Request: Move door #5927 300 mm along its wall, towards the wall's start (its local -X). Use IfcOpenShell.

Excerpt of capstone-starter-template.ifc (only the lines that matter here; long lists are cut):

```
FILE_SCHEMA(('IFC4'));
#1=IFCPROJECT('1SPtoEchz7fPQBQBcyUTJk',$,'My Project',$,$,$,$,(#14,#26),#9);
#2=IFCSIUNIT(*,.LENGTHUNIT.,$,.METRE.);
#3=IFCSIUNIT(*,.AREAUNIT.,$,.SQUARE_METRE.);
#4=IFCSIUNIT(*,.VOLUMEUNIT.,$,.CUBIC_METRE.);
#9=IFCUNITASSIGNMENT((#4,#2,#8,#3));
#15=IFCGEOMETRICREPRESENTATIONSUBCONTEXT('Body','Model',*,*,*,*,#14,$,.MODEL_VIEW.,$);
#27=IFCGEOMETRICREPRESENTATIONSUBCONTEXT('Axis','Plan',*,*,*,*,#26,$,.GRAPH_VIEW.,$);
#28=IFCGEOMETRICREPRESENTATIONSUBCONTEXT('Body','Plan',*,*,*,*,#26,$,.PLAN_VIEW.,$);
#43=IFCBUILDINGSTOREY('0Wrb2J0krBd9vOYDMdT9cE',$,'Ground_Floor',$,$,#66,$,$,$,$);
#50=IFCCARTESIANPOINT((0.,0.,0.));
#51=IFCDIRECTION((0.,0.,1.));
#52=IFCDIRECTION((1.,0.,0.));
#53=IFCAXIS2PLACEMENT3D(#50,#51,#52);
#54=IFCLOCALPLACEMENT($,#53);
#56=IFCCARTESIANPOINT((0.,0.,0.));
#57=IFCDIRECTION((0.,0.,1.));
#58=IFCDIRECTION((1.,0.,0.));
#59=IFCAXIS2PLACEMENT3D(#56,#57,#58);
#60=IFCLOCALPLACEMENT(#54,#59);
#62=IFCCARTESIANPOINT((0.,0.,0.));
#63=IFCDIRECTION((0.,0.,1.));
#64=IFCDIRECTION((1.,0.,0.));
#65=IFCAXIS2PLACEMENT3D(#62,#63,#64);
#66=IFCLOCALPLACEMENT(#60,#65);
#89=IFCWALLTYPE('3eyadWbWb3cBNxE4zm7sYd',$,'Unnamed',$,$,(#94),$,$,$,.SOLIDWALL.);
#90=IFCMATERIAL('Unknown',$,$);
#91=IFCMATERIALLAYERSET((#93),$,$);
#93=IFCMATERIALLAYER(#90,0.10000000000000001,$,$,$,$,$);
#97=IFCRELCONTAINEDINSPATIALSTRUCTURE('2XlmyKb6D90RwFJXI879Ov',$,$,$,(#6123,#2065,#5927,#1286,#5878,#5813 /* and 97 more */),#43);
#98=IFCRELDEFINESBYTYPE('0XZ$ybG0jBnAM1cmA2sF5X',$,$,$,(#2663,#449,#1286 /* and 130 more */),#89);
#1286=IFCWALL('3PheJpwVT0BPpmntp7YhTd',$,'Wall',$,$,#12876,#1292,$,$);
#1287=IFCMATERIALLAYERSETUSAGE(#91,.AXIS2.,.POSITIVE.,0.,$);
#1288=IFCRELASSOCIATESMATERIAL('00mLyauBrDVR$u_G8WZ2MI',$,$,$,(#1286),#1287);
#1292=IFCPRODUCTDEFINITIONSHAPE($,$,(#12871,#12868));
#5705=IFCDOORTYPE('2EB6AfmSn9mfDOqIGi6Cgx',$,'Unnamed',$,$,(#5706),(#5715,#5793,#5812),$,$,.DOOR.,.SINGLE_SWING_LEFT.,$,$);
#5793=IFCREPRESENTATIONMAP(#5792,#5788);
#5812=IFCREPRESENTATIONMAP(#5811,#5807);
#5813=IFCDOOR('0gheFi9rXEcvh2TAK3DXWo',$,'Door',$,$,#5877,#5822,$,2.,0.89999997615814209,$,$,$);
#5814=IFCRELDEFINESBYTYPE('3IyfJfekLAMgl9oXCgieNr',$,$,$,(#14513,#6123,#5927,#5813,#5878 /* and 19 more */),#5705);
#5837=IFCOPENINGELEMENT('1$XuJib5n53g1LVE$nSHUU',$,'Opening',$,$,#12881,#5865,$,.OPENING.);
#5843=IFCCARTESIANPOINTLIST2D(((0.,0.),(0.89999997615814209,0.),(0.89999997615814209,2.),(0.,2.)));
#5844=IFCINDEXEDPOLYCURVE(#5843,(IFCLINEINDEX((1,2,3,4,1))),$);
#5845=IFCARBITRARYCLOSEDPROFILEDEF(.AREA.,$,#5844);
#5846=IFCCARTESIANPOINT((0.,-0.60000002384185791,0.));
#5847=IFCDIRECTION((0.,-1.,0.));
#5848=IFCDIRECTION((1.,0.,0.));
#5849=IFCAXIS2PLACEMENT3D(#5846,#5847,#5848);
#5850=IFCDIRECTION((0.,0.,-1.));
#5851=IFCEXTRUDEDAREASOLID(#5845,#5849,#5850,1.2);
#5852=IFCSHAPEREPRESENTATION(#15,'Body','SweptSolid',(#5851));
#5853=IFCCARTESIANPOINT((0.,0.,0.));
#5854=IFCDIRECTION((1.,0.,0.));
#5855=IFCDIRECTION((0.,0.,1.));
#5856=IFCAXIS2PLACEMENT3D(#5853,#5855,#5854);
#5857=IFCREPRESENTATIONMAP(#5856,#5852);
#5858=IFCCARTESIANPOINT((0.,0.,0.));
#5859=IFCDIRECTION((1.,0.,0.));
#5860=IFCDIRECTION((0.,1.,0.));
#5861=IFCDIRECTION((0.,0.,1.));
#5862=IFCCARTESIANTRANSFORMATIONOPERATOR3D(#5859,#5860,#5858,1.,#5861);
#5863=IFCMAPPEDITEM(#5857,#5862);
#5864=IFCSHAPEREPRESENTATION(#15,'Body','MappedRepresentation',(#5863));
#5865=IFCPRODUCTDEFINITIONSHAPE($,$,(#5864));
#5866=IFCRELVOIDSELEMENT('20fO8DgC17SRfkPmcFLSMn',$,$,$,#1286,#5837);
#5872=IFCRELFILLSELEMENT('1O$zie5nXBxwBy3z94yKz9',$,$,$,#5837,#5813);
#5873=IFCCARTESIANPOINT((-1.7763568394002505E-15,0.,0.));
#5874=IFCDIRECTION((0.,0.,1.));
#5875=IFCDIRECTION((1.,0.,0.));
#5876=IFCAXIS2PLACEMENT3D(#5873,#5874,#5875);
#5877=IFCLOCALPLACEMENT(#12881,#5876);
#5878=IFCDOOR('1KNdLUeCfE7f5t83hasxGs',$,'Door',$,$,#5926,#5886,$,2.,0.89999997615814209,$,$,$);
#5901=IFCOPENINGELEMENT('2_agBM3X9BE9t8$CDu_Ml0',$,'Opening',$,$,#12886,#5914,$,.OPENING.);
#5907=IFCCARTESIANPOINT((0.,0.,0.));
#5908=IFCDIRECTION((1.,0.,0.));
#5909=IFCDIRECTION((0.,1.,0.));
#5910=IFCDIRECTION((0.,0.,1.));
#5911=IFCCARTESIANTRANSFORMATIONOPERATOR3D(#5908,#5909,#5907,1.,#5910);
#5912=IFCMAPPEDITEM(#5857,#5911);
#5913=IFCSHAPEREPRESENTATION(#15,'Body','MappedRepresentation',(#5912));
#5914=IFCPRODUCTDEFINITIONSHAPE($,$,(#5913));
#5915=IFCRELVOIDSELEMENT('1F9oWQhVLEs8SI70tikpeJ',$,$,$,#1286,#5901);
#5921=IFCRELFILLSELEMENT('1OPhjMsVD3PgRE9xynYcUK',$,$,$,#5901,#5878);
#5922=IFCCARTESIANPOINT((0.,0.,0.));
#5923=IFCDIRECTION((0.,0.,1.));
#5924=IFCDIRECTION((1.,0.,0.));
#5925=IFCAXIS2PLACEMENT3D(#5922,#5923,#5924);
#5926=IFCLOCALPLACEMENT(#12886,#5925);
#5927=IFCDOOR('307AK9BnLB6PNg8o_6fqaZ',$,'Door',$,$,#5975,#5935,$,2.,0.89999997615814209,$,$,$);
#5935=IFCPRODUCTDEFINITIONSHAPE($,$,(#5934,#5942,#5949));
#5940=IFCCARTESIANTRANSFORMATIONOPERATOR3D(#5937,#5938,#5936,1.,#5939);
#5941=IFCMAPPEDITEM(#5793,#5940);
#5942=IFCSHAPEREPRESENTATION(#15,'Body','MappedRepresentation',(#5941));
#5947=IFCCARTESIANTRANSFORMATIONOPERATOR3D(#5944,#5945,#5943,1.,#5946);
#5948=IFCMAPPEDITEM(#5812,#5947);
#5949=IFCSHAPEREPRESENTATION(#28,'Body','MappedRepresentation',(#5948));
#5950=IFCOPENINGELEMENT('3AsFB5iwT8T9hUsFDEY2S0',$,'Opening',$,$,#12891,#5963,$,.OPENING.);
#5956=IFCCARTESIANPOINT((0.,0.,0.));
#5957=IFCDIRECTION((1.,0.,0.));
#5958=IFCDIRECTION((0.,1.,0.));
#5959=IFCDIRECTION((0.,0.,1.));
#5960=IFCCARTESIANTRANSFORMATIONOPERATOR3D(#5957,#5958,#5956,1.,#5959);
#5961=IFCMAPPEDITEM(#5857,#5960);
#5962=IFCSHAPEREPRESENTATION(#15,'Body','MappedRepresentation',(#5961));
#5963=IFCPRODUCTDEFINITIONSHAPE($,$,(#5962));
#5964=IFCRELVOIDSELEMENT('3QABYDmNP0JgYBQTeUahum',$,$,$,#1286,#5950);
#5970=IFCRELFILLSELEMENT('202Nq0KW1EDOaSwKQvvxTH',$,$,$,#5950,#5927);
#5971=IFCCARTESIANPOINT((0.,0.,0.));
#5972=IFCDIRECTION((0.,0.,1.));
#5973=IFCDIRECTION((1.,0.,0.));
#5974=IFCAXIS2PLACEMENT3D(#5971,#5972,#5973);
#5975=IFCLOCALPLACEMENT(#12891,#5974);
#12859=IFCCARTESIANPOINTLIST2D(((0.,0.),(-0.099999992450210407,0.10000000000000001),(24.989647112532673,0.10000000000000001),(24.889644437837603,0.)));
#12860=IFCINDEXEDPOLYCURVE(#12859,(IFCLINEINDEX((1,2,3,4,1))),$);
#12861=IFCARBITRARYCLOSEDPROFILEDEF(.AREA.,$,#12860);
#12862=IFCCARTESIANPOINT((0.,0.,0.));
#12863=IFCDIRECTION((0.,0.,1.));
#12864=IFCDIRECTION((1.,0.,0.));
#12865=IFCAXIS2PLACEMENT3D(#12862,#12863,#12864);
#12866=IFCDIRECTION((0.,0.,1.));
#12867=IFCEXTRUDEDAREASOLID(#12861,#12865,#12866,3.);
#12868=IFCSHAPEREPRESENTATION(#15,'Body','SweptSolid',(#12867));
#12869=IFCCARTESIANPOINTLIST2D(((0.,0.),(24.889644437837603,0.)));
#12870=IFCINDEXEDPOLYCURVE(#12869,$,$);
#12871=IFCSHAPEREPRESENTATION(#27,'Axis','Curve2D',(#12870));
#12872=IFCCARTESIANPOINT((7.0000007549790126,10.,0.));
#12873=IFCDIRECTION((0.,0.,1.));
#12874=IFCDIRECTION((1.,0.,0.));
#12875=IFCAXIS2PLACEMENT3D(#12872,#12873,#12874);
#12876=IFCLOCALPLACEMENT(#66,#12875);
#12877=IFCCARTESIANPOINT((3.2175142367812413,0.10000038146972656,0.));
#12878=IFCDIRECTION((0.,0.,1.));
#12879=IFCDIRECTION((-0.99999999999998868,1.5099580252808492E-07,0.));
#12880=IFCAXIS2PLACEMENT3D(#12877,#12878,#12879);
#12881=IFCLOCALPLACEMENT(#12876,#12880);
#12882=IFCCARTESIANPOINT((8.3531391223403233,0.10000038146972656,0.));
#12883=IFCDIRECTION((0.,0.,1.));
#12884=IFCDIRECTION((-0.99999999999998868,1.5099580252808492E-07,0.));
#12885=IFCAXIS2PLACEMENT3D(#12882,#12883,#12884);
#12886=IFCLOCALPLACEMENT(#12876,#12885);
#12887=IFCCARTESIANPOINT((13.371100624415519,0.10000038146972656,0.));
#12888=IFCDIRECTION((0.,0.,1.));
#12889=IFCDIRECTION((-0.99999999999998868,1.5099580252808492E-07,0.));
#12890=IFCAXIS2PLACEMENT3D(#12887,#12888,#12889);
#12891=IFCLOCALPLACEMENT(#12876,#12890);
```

```python
import ifcopenshell
import ifcopenshell.api.geometry
import ifcopenshell.util.placement

model = ifcopenshell.open("capstone-starter-template.ifc")

door = model.by_guid("307AK9BnLB6PNg8o_6fqaZ")
opening = door.FillsVoids[0].RelatingOpeningElement
wall = opening.VoidsElements[0].RelatingBuildingElement

wall_matrix = ifcopenshell.util.placement.get_local_placement(wall.ObjectPlacement)
shift = wall_matrix[:3, 0] * -0.3
before = ifcopenshell.util.placement.get_local_placement(door.ObjectPlacement)[:3, 3].copy()

# The door is placed relative to its opening, so it follows when the opening moves.
matrix = ifcopenshell.util.placement.get_local_placement(opening.ObjectPlacement)
matrix[:3, 3] += shift
ifcopenshell.api.geometry.edit_object_placement(
    model, product=opening, matrix=matrix, is_si=False, should_transform_children=True
)

after = ifcopenshell.util.placement.get_local_placement(door.ObjectPlacement)[:3, 3]
print("door moved by", (after - before).round(3) + 0.0)

model.write("capstone-starter-template_edited.ifc")
```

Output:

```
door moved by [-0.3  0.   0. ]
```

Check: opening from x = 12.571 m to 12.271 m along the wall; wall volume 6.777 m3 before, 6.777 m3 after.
